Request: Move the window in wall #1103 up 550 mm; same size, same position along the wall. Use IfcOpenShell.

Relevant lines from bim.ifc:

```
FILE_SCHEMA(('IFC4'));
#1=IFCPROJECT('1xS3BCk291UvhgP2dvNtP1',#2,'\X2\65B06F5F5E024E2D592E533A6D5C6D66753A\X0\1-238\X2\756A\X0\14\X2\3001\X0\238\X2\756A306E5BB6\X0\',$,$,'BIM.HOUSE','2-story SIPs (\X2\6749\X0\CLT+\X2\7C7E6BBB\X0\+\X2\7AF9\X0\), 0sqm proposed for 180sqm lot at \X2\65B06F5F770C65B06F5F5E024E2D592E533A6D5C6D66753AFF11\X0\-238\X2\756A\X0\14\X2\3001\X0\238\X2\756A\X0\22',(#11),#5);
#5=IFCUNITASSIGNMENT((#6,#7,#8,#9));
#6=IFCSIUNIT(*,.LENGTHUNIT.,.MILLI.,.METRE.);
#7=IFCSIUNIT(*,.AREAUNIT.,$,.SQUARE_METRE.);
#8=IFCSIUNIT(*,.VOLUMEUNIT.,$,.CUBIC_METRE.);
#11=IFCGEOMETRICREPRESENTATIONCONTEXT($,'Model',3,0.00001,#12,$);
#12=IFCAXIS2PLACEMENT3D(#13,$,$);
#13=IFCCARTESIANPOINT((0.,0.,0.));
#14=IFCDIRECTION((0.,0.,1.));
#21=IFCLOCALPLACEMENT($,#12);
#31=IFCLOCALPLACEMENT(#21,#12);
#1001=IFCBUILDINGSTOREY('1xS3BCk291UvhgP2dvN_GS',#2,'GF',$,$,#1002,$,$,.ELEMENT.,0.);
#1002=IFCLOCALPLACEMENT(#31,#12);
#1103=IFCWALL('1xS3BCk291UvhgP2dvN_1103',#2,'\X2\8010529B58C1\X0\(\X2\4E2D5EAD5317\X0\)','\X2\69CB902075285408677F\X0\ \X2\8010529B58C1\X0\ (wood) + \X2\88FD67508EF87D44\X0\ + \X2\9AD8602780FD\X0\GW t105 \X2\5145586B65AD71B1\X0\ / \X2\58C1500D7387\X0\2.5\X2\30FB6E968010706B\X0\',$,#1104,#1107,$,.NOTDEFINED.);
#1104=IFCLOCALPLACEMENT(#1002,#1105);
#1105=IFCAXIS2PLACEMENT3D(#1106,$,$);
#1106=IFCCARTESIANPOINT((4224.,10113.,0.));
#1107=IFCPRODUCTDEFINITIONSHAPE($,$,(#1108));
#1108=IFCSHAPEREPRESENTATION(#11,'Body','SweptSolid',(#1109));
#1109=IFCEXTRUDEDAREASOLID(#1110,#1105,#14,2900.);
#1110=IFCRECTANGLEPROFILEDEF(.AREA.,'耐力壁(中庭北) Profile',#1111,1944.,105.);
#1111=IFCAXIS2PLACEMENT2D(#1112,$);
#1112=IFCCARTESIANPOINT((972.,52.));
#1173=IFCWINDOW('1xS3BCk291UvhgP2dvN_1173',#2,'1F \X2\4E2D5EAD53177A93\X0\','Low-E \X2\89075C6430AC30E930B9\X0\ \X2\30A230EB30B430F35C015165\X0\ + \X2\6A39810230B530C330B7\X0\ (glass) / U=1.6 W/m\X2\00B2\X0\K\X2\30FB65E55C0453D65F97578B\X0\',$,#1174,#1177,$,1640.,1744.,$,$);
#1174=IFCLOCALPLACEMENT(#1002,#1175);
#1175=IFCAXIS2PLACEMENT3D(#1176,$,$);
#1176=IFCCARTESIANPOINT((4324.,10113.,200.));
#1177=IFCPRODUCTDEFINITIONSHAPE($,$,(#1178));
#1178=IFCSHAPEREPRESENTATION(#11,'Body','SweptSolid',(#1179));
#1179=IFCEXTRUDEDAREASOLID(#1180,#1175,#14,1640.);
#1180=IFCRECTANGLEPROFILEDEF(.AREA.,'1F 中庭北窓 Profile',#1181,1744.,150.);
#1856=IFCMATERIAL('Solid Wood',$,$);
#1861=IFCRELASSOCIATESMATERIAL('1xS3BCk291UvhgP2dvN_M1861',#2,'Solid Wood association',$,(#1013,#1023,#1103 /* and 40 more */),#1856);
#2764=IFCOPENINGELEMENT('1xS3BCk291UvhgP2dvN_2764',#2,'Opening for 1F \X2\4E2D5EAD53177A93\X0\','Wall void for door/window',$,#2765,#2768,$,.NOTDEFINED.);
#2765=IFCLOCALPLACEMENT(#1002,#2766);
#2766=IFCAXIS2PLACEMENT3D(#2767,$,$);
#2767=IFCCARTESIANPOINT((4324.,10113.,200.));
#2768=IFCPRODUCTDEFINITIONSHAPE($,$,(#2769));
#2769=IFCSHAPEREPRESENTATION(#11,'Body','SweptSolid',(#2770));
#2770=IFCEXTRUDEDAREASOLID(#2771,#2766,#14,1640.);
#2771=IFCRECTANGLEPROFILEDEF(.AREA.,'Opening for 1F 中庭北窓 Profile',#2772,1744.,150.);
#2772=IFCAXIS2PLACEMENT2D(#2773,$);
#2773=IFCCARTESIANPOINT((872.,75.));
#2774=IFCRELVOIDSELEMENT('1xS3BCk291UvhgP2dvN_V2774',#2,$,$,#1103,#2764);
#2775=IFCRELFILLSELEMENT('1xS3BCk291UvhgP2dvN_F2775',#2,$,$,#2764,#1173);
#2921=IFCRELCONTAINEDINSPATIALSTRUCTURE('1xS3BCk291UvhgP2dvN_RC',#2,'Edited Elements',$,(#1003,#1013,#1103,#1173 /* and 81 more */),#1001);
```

```python
import numpy as np
import ifcopenshell
import ifcopenshell.api.geometry
import ifcopenshell.util.placement
import ifcopenshell.util.unit

model = ifcopenshell.open("bim.ifc")
unit_scale = ifcopenshell.util.unit.calculate_unit_scale(model)

window = model.by_id(1173)
opening = window.FillsVoids[0].RelatingOpeningElement
dz = 550.0

shift = np.array([0.0, 0.0, dz])
# The window is not placed relative to its opening, so move both.
for product in (opening, window):
    matrix = ifcopenshell.util.placement.get_local_placement(product.ObjectPlacement)
    matrix[:3, 3] += shift
    ifcopenshell.api.geometry.edit_object_placement(model, product=product, matrix=matrix, is_si=False)

print(f"moved by {dz * unit_scale:+.3f} m")

model.write("bim_v2.ifc")
```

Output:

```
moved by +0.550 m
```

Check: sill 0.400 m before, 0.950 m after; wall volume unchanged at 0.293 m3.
